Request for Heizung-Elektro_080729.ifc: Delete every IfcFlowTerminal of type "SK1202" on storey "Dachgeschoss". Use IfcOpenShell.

First a look at what the model holds.

```python
import ifcopenshell
import ifcopenshell.util.element

model = ifcopenshell.open("Heizung-Elektro_080729.ifc")
print(model.schema)
storey = next(s for s in model.by_type("IfcBuildingStorey") if s.Name == "Dachgeschoss")
terminals = [e for e in ifcopenshell.util.element.get_decomposition(storey) if e.is_a("IfcFlowTerminal")]
seen = {}
for e in terminals:
    element_type = ifcopenshell.util.element.get_type(e)
    name = element_type.Name if element_type not in (None, e) else None
    seen[name] = seen.get(name, 0) + 1
for name, count in sorted(seen.items(), key=str):
    print(count, "x", name)
```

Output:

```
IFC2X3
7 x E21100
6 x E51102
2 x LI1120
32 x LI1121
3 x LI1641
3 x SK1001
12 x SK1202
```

```python
import ifcopenshell
import ifcopenshell.api.root
import ifcopenshell.util.element

model = ifcopenshell.open("Heizung-Elektro_080729.ifc")

storey = next(s for s in model.by_type("IfcBuildingStorey") if s.Name == "Dachgeschoss")
terminals = [e for e in ifcopenshell.util.element.get_decomposition(storey) if e.is_a("IfcFlowTerminal")]
targets = [e for e in terminals if (t := ifcopenshell.util.element.get_type(e)) not in (None, e) and t.Name == "SK1202"]

for e in targets:
    ifcopenshell.api.root.remove_product(model, product=e)
print(len(targets), "removed")

model.write("Heizung-Elektro_080729_rev.ifc")
```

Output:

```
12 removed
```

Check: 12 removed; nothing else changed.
